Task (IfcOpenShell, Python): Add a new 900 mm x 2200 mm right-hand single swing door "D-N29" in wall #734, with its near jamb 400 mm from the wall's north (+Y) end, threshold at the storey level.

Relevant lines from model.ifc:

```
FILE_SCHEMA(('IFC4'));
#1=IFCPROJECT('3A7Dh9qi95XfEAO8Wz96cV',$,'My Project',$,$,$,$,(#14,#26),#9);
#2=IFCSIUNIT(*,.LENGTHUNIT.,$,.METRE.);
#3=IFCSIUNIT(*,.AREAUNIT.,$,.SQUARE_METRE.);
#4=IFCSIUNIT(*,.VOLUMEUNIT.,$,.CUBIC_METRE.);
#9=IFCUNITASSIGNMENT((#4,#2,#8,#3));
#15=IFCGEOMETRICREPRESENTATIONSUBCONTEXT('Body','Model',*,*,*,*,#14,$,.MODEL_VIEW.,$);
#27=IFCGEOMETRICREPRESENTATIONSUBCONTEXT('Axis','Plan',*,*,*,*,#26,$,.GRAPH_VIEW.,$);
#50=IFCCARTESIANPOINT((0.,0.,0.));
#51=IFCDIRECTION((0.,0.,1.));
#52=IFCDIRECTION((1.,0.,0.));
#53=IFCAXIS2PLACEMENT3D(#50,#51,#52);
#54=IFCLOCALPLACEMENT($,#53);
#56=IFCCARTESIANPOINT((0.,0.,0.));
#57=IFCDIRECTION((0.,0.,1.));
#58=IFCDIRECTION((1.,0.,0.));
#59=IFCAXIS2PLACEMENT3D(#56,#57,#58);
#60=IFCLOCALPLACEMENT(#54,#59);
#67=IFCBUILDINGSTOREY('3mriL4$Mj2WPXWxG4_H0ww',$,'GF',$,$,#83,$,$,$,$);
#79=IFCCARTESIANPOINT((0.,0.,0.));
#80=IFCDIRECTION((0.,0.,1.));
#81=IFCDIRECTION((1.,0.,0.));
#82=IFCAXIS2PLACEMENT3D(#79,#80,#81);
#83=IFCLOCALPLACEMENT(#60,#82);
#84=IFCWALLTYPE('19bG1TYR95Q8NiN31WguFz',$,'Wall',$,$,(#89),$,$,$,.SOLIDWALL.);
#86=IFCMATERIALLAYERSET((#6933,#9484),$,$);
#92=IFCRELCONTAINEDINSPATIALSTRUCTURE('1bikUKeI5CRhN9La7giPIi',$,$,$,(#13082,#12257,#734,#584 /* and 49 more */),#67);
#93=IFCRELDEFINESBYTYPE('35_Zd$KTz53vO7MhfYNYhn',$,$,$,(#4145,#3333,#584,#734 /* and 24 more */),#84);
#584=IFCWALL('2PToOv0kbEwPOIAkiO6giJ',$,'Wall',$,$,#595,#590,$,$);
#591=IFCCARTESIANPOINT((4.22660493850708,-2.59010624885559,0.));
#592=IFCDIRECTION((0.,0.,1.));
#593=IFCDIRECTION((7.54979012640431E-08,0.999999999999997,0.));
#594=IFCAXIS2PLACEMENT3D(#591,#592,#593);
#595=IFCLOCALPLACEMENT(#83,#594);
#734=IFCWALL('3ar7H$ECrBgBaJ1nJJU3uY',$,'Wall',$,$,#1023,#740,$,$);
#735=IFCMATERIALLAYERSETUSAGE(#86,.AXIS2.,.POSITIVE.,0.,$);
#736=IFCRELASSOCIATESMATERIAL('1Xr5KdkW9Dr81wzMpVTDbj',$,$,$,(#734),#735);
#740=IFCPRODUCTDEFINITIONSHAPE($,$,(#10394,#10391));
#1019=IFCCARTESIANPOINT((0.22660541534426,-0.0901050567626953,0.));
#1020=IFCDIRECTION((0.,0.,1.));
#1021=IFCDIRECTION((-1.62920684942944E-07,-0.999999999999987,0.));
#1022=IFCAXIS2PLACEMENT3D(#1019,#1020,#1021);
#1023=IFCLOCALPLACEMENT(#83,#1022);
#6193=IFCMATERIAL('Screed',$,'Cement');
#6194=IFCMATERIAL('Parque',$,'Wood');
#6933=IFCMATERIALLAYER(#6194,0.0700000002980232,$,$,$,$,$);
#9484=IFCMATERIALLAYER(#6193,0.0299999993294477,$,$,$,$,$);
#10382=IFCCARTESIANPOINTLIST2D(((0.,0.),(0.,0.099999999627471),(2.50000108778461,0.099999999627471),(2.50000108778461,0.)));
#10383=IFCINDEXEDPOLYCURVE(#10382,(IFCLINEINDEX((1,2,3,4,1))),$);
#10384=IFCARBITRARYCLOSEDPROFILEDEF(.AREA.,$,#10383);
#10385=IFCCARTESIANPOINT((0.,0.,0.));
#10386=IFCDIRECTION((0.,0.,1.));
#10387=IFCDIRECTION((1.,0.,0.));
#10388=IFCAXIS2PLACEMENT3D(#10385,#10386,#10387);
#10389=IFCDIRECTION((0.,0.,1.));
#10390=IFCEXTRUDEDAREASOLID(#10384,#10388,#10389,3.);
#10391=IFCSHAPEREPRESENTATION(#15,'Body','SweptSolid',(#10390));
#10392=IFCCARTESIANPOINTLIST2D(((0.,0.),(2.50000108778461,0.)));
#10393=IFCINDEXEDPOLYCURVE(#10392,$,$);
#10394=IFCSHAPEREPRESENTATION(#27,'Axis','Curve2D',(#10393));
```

```python
import numpy as np
import ifcopenshell
import ifcopenshell.api.feature
import ifcopenshell.api.geometry
import ifcopenshell.api.root
import ifcopenshell.api.spatial
import ifcopenshell.geom
import ifcopenshell.util.element
import ifcopenshell.util.placement
import ifcopenshell.util.representation
import ifcopenshell.util.shape
import ifcopenshell.util.unit

model = ifcopenshell.open("model.ifc")
unit_scale = ifcopenshell.util.unit.calculate_unit_scale(model)
settings = ifcopenshell.geom.settings()


def volume(element):
    """Net volume in cubic metres, openings subtracted."""
    shape = ifcopenshell.geom.create_shape(settings, element)
    return ifcopenshell.util.shape.get_volume(shape.geometry)


wall = model.by_guid("3ar7H$ECrBgBaJ1nJJU3uY")
storey = ifcopenshell.util.element.get_container(wall, ifc_class="IfcBuildingStorey")
context = ifcopenshell.util.representation.get_context(model, "Model", "Body", "MODEL_VIEW")
before = volume(wall)

width, height, from_end, sill = 0.9, 2.2, 0.4, 0.0  # metres

# The wall runs along its own X axis, and the end named is its -X end.
wall_shape = ifcopenshell.geom.create_shape(settings, wall)
x, y, z = ifcopenshell.util.shape.get_vertices(wall_shape.geometry).T
start = x.min() + from_end
face, thickness = float(y.min()), float(y.max() - y.min())
wall_matrix = ifcopenshell.util.placement.get_local_placement(wall.ObjectPlacement)
level = ifcopenshell.util.placement.get_local_placement(storey.ObjectPlacement)[2, 3]


def in_wall(x, y):
    """Placement at x, y metres in the wall's axes, at sill height."""
    matrix = wall_matrix.copy()
    matrix[:, 3] = wall_matrix @ np.array([x / unit_scale, y / unit_scale, 0.0, 1.0])
    matrix[2, 3] = level + sill / unit_scale
    return matrix


# Opening: a box that overshoots both wall faces by 50 mm.
opening = ifcopenshell.api.root.create_entity(model, ifc_class="IfcOpeningElement", predefined_type="OPENING")
box = ifcopenshell.api.geometry.add_wall_representation(
    model, context=context, length=width, height=height, thickness=thickness + 0.1
)
ifcopenshell.api.geometry.assign_representation(model, product=opening, representation=box)
ifcopenshell.api.geometry.edit_object_placement(model, product=opening, matrix=in_wall(start, face - 0.05), is_si=False)
ifcopenshell.api.feature.add_feature(model, feature=opening, element=wall)

door = ifcopenshell.api.root.create_entity(model, ifc_class="IfcDoor", name="D-N29", predefined_type="DOOR")
door.OverallWidth, door.OverallHeight = width / unit_scale, height / unit_scale
door.OperationType = "SINGLE_SWING_RIGHT"
body = ifcopenshell.api.geometry.add_door_representation(
    model,
    context=context,
    overall_width=door.OverallWidth,
    overall_height=door.OverallHeight,
    operation_type="SINGLE_SWING_RIGHT",
    lining_properties={"LiningDepth": thickness / unit_scale, "ThresholdDepth": thickness / unit_scale},
)
ifcopenshell.api.geometry.assign_representation(model, product=door, representation=body)
ifcopenshell.api.spatial.assign_container(model, products=[door], relating_structure=storey)
ifcopenshell.api.feature.add_filling(model, opening=opening, element=door)

# The lining spans the wall, so the door starts at the wall face.
ifcopenshell.api.geometry.edit_object_placement(model, product=door, matrix=in_wall(start, face), is_si=False)

after = volume(wall)

print(f"wall volume {before:.3f} -> {after:.3f} m3")

model.write("model_updated.ifc")
```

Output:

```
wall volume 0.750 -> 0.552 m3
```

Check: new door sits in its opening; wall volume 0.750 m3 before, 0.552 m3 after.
